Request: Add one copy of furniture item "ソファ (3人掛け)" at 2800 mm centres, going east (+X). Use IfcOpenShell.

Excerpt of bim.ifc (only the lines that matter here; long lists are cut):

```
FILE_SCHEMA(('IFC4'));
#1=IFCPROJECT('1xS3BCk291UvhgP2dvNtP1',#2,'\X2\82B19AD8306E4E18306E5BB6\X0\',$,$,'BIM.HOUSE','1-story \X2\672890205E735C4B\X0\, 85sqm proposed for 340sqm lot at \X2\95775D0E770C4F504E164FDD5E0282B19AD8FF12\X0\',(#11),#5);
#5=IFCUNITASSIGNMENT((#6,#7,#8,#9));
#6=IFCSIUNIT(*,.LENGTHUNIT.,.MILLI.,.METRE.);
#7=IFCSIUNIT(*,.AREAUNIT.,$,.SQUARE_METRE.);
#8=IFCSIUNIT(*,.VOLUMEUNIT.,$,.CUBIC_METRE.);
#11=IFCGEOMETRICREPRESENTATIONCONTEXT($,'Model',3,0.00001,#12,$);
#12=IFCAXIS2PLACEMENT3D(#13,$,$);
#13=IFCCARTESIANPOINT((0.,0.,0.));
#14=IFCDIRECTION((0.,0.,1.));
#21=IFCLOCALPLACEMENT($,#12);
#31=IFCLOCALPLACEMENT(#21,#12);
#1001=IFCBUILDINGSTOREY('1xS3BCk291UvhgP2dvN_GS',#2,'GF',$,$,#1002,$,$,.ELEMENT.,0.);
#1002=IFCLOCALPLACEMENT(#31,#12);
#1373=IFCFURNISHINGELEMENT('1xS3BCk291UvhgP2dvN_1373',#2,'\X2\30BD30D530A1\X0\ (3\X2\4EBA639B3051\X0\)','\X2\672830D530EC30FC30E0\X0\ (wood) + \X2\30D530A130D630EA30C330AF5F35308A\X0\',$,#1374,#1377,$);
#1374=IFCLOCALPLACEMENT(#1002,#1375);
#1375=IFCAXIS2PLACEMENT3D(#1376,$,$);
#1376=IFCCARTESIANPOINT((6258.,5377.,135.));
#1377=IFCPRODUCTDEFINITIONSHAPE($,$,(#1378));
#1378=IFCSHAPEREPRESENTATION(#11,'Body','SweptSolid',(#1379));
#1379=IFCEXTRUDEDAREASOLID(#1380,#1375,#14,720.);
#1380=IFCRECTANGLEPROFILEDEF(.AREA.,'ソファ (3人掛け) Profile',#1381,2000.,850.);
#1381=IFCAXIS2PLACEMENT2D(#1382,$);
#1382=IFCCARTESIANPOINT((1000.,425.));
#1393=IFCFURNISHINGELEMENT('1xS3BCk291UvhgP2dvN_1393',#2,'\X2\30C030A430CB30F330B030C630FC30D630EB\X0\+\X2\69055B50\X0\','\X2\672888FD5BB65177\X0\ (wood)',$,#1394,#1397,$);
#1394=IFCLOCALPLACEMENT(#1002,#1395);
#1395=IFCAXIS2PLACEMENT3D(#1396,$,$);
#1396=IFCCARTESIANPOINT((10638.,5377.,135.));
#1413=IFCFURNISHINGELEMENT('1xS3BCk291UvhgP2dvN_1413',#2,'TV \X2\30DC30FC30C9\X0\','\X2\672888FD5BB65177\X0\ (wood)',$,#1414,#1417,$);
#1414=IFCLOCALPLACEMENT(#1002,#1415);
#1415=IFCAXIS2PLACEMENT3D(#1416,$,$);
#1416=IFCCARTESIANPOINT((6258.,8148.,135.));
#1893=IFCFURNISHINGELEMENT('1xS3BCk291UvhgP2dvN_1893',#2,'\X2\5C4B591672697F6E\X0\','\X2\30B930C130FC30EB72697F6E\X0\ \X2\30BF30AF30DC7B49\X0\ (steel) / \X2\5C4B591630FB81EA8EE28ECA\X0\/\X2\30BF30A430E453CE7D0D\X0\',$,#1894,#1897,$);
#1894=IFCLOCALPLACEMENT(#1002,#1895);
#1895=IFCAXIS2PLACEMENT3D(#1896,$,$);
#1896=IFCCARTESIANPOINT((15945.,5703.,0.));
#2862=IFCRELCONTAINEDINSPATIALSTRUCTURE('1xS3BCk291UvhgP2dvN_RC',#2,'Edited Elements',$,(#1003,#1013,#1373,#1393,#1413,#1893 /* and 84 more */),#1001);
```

```python
import numpy as np
import ifcopenshell
import ifcopenshell.api.geometry
import ifcopenshell.api.root
import ifcopenshell.util.element
import ifcopenshell.util.placement
import ifcopenshell.util.unit

model = ifcopenshell.open("bim.ifc")
unit_scale = ifcopenshell.util.unit.calculate_unit_scale(model)


def reuse_history(source, copy):
    """copy_class also copies each property set's owner history, people and application; keep the originals."""
    for rel in copy.IsDefinedBy:
        if rel.is_a("IfcRelDefinesByProperties") and (history := rel.RelatingPropertyDefinition.OwnerHistory):
            rel.RelatingPropertyDefinition.OwnerHistory = source.OwnerHistory
            ifcopenshell.util.element.remove_deep2(model, history)


source = model.by_guid("1xS3BCk291UvhgP2dvN_1373")
base = ifcopenshell.util.placement.get_local_placement(source.ObjectPlacement)
step = np.array([1.0, 0.0, 0.0]) * 2.8 / unit_scale

for i in range(1, 2):
    copy = ifcopenshell.api.root.copy_class(model, product=source)
    copy.Representation = ifcopenshell.util.element.copy_deep(
        model, source.Representation, exclude=["IfcGeometricRepresentationContext", "IfcRepresentationMap"]
    )
    reuse_history(source, copy)
    matrix = base.copy()
    matrix[:3, 3] += i * step
    print("added at", matrix[:3, 3].round(3) + 0.0)
    ifcopenshell.api.geometry.edit_object_placement(model, product=copy, matrix=matrix, is_si=False)

model.write("bim_edited.ifc")
```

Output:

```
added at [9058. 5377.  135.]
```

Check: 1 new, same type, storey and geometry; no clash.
